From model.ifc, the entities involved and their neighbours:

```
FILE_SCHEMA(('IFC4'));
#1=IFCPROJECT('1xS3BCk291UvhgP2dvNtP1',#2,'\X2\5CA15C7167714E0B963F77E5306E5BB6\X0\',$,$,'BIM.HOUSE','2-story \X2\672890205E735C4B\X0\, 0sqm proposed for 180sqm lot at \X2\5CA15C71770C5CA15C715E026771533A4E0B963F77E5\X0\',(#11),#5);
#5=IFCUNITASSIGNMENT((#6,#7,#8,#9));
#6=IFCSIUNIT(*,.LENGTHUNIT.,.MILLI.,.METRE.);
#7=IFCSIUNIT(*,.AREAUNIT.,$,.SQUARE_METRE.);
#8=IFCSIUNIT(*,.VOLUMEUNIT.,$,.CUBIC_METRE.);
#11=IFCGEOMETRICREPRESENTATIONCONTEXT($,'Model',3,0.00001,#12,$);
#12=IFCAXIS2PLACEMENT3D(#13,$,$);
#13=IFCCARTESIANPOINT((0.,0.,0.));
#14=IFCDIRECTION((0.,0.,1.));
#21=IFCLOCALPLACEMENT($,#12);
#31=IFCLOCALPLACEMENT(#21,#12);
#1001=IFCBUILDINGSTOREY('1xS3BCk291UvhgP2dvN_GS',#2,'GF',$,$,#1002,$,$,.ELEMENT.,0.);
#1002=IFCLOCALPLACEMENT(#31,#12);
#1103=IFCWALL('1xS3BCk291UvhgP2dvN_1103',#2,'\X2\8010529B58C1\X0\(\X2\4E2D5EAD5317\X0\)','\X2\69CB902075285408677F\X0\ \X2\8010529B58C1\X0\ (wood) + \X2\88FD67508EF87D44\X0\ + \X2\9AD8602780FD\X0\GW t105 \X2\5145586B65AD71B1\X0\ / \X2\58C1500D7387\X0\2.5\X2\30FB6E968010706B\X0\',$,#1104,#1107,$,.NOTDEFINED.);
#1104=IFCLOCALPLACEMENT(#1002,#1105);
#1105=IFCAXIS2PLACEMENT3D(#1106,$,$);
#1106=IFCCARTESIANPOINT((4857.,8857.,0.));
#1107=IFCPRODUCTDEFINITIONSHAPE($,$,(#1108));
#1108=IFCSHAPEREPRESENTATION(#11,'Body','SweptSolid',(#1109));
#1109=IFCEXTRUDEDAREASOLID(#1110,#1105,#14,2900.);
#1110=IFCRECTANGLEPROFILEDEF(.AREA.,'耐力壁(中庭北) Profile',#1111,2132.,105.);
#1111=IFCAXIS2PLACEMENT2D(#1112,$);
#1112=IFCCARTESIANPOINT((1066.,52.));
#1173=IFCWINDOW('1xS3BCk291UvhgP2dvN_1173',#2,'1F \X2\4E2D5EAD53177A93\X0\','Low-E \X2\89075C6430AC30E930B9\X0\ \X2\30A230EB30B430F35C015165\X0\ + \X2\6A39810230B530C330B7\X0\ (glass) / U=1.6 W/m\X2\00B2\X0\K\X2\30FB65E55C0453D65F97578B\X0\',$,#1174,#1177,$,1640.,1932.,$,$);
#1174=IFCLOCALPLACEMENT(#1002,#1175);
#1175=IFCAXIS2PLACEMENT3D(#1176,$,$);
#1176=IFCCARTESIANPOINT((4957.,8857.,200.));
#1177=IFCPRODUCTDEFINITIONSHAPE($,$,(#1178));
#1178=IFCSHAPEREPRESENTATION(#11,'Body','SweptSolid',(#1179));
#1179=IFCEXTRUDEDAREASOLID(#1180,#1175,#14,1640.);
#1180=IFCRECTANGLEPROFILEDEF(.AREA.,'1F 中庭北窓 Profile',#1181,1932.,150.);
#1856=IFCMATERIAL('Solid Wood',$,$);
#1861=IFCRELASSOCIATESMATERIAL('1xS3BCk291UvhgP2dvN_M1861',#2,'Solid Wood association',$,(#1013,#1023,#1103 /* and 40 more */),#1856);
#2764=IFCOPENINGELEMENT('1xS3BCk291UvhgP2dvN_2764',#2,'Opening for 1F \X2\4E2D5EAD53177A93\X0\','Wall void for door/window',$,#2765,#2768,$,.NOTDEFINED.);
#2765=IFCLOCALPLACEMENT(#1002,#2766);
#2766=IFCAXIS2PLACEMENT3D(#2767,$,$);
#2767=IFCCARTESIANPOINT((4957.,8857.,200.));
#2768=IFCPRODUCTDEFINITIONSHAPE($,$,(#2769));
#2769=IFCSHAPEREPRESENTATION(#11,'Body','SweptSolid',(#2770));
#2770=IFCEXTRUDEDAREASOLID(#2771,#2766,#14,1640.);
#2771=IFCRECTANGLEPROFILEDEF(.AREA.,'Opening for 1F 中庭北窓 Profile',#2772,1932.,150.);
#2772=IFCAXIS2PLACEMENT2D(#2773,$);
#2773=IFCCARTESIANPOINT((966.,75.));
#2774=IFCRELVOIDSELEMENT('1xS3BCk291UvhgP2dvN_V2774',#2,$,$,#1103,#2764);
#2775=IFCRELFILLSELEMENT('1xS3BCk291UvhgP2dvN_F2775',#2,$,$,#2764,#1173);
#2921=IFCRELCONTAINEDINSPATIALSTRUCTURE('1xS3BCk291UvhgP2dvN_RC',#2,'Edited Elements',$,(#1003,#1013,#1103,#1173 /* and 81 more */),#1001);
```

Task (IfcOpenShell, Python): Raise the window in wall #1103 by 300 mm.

```python
import numpy as np
import ifcopenshell
import ifcopenshell.api.geometry
import ifcopenshell.util.placement
import ifcopenshell.util.unit

model = ifcopenshell.open("model.ifc")
unit_scale = ifcopenshell.util.unit.calculate_unit_scale(model)

window = model.by_id(1173)
opening = window.FillsVoids[0].RelatingOpeningElement
dz = 0.3 / unit_scale

shift = np.array([0.0, 0.0, dz])
# The window is not placed relative to its opening, so move both.
for product in (opening, window):
    matrix = ifcopenshell.util.placement.get_local_placement(product.ObjectPlacement)
    matrix[:3, 3] += shift
    ifcopenshell.api.geometry.edit_object_placement(model, product=product, matrix=matrix, is_si=False)

print(f"moved by {dz * unit_scale:+.3f} m")

model.write("model-out.ifc")
```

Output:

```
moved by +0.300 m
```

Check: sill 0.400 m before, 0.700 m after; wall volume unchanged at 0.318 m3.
